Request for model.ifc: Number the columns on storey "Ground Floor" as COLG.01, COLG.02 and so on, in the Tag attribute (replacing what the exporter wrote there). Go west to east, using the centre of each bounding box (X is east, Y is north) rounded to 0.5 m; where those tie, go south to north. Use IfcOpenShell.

First a look at what the model holds.

```python
import ifcopenshell
import ifcopenshell.util.element
import ifcopenshell.util.placement

model = ifcopenshell.open("model.ifc")
print(model.schema)
storey = next(s for s in model.by_type("IfcBuildingStorey") if s.Name == "Ground Floor")
columns = [e for e in ifcopenshell.util.element.get_decomposition(storey) if e.is_a("IfcColumn")]
for e in sorted(columns, key=lambda e: e.id()):
    origin = ifcopenshell.util.placement.get_local_placement(e.ObjectPlacement)[:3, 3]
    print(e.id(), e.Tag, e.Name, origin.round(2) + 0.0, sep=" | ")
```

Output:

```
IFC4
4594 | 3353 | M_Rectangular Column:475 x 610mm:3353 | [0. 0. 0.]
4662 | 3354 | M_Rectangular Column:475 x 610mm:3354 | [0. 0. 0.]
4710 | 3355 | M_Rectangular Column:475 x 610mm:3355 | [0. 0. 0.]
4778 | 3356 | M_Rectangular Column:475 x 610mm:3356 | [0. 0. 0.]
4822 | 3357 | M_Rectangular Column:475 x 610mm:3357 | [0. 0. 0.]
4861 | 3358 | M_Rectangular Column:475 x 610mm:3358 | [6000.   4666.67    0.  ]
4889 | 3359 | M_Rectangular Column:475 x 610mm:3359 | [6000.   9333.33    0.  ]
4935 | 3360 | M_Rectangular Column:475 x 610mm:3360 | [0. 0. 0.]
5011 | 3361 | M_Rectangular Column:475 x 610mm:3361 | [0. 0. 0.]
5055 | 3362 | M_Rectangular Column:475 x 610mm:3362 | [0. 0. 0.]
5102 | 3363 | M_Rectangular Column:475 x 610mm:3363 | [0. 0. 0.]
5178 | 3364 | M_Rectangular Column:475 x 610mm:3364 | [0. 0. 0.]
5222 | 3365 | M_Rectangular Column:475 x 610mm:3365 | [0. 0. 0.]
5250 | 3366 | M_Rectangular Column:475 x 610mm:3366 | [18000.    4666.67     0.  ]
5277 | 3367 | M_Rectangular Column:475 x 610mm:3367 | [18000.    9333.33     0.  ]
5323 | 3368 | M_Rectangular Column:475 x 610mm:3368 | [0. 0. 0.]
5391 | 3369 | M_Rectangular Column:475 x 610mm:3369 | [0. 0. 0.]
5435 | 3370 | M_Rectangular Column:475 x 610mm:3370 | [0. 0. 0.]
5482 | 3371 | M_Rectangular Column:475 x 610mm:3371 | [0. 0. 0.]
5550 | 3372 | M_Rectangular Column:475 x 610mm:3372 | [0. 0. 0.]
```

```python
import ifcopenshell
import ifcopenshell.geom
import ifcopenshell.util.element
import ifcopenshell.util.shape

model = ifcopenshell.open("model.ifc")
settings = ifcopenshell.geom.settings()
settings.set("use-world-coords", True)


def centre(element):
    shape = ifcopenshell.geom.create_shape(settings, element)
    return ifcopenshell.util.shape.get_bbox_centroid(shape.geometry)


storey = next(s for s in model.by_type("IfcBuildingStorey") if s.Name == "Ground Floor")
columns = [e for e in ifcopenshell.util.element.get_decomposition(storey) if e.is_a("IfcColumn")]

# Insertion points can sit at a corner or the storey origin, so sort by the geometry (in metres).
centres = {e: centre(e) for e in columns}
columns.sort(key=lambda e: (round(centres[e][0] / 0.5), centres[e][1]))

for i, e in enumerate(columns, start=1):
    number = f"COLG.{i:02d}"
    e.Tag = number
    print(e.id(), number)

model.write("model_v2.ifc")
```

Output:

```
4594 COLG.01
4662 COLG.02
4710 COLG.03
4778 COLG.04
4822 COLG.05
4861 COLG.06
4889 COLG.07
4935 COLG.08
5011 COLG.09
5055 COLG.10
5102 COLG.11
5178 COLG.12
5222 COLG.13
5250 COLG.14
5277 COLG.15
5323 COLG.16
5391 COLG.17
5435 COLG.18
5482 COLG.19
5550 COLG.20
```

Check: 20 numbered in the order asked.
